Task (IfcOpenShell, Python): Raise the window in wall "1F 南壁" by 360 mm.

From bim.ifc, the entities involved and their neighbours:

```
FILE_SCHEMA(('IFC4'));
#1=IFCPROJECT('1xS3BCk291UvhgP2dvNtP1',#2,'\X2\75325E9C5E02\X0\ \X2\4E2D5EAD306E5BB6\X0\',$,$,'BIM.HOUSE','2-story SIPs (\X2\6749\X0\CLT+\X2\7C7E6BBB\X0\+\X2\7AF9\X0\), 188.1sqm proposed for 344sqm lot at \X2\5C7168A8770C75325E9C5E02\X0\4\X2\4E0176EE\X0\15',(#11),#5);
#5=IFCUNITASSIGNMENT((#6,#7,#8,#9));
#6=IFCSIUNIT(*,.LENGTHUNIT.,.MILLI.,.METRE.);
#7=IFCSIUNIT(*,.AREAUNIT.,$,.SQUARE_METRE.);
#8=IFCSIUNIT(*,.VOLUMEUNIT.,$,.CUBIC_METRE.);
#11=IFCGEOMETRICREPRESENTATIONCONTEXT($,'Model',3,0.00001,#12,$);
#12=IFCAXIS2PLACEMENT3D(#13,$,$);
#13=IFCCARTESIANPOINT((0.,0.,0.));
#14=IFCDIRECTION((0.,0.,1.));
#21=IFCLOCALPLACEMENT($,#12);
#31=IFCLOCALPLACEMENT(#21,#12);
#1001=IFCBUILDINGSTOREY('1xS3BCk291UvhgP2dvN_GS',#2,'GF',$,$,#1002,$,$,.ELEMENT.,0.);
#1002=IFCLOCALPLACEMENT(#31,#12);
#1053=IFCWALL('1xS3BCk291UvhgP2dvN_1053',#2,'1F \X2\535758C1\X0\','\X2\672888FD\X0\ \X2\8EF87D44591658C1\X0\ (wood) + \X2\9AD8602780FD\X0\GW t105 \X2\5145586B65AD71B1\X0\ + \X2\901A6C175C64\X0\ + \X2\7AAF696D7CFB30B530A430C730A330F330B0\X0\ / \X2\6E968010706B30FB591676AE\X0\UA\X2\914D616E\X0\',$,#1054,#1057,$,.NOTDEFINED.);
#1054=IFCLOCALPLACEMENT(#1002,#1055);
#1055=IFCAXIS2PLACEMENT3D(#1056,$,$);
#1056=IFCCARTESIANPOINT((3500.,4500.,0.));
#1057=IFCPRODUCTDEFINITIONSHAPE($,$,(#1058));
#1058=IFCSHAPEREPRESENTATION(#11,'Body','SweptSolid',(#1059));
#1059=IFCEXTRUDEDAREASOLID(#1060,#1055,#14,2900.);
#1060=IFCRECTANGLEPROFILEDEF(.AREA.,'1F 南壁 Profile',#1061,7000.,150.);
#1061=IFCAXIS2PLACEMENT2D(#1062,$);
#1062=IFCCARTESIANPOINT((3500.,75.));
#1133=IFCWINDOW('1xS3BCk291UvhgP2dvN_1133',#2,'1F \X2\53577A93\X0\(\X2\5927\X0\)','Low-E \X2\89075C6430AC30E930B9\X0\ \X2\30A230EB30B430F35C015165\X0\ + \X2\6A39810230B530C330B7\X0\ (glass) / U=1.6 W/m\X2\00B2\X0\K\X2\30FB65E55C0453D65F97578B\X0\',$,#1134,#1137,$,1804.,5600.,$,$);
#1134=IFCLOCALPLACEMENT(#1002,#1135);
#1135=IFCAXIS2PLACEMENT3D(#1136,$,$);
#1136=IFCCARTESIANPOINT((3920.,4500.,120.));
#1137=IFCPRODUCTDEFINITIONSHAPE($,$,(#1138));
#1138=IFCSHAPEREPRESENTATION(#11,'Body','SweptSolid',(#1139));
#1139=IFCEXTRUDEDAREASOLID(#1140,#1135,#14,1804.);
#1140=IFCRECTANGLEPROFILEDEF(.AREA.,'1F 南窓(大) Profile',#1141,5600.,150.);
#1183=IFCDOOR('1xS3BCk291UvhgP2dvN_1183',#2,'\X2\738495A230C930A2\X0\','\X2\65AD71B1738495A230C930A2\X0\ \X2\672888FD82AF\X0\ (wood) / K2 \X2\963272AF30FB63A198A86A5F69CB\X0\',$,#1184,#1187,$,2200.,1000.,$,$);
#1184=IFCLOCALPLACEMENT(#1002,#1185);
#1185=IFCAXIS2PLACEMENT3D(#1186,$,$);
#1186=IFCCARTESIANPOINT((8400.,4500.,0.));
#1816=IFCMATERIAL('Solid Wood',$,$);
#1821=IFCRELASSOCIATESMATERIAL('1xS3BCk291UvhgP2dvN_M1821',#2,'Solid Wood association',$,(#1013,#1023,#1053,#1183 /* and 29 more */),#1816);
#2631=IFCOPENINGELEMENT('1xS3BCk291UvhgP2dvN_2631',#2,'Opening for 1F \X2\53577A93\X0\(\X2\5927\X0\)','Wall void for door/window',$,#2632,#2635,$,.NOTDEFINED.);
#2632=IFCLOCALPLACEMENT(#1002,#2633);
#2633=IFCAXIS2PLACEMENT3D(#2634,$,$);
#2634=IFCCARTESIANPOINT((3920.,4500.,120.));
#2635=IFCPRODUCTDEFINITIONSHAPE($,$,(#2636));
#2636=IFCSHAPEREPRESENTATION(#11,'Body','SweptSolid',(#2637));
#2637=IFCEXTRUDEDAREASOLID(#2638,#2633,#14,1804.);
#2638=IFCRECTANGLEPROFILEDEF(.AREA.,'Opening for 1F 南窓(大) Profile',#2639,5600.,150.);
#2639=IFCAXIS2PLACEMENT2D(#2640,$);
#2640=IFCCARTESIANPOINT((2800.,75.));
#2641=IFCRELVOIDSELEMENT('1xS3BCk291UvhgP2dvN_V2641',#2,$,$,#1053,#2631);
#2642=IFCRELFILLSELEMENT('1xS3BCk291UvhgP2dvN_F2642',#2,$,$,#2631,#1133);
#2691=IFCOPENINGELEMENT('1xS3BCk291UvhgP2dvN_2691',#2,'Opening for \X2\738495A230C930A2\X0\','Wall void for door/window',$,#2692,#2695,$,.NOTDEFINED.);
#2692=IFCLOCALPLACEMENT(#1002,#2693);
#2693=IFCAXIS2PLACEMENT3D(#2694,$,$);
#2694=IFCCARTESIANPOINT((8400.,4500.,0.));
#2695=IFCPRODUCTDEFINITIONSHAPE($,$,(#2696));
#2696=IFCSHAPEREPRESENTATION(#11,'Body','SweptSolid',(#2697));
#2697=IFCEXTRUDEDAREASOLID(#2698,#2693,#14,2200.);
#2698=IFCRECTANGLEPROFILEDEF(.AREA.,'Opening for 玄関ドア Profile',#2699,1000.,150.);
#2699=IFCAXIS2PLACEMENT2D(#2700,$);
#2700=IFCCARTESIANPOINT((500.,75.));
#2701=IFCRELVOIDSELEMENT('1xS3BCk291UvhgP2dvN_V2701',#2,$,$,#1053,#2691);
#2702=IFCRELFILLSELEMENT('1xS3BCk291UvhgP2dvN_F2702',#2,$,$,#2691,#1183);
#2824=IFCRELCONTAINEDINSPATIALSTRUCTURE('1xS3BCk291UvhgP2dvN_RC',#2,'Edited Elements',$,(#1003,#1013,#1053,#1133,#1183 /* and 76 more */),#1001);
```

```python
import numpy as np
import ifcopenshell
import ifcopenshell.api.geometry
import ifcopenshell.util.placement
import ifcopenshell.util.unit

model = ifcopenshell.open("bim.ifc")
unit_scale = ifcopenshell.util.unit.calculate_unit_scale(model)

window = model.by_guid("1xS3BCk291UvhgP2dvN_1133")
opening = window.FillsVoids[0].RelatingOpeningElement
dz = 360.0

shift = np.array([0.0, 0.0, dz])
# The window is not placed relative to its opening, so move both.
for product in (opening, window):
    matrix = ifcopenshell.util.placement.get_local_placement(product.ObjectPlacement)
    matrix[:3, 3] += shift
    ifcopenshell.api.geometry.edit_object_placement(model, product=product, matrix=matrix, is_si=False)

print(f"moved by {dz * unit_scale:+.3f} m")

model.write("bim_v2.ifc")
```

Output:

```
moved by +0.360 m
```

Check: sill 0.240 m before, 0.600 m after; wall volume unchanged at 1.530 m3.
